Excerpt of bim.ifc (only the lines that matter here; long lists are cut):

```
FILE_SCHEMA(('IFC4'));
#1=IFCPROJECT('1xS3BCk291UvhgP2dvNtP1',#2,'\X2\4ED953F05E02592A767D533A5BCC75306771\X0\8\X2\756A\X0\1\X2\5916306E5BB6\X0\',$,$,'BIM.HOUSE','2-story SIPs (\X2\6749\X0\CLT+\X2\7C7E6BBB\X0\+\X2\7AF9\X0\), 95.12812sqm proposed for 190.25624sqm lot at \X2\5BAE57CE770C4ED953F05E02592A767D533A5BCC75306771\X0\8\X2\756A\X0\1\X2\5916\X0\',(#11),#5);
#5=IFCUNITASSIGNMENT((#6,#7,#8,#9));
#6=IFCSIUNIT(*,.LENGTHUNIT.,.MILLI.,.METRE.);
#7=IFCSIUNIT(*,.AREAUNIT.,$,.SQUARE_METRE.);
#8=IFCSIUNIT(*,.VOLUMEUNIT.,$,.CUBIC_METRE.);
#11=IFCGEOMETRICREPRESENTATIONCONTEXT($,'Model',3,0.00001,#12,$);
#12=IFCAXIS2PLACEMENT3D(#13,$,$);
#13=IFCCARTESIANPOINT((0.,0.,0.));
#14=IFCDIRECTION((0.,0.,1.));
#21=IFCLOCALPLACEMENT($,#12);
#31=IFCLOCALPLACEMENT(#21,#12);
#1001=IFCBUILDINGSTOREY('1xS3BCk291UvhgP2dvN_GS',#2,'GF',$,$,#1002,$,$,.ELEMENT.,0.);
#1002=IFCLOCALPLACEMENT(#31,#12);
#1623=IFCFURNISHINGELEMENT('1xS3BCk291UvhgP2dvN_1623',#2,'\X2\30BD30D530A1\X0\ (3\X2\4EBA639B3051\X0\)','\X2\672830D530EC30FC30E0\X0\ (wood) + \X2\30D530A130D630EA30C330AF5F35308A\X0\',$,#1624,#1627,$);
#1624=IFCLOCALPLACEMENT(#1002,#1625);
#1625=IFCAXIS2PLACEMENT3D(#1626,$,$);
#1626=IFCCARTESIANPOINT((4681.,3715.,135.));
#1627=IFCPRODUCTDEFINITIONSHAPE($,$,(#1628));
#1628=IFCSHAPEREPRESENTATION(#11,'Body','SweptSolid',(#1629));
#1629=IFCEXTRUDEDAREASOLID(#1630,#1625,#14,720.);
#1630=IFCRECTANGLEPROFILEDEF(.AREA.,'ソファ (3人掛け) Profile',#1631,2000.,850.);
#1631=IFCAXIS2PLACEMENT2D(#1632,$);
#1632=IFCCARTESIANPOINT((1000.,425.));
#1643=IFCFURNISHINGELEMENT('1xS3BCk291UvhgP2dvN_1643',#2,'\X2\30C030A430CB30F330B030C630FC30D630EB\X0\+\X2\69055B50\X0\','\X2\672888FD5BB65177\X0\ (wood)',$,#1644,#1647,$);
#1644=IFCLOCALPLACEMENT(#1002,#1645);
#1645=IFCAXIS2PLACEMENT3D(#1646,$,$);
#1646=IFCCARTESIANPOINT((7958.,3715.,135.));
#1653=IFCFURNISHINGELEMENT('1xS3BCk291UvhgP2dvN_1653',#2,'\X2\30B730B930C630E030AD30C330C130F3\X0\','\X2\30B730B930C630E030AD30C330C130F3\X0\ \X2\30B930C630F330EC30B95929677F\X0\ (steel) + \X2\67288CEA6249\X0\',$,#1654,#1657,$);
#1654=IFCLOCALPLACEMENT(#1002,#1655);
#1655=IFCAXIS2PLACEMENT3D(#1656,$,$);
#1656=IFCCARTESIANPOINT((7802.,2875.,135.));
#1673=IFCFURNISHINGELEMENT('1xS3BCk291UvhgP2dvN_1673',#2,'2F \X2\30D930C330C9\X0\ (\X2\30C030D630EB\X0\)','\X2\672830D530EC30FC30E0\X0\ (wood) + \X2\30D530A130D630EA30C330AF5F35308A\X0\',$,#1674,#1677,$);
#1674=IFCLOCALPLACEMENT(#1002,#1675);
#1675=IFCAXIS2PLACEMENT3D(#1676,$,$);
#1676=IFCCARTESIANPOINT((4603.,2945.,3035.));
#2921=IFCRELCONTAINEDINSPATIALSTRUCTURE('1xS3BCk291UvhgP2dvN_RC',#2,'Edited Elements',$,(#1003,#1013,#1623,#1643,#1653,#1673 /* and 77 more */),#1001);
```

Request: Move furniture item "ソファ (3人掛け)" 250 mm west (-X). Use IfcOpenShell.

```python
import ifcopenshell
import ifcopenshell.api.geometry
import ifcopenshell.util.placement

model = ifcopenshell.open("bim.ifc")

item = model.by_guid("1xS3BCk291UvhgP2dvN_1623")
matrix = ifcopenshell.util.placement.get_local_placement(item.ObjectPlacement)
matrix[0, 3] -= 250.0
ifcopenshell.api.geometry.edit_object_placement(model, product=item, matrix=matrix, is_si=False)

print(ifcopenshell.util.placement.get_local_placement(item.ObjectPlacement).round(3) + 0.0)

model.write("bim_rev.ifc")
```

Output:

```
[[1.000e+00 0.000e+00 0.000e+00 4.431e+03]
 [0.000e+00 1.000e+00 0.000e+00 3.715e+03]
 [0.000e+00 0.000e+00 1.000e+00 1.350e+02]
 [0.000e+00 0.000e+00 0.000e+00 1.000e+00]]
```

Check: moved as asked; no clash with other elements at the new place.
